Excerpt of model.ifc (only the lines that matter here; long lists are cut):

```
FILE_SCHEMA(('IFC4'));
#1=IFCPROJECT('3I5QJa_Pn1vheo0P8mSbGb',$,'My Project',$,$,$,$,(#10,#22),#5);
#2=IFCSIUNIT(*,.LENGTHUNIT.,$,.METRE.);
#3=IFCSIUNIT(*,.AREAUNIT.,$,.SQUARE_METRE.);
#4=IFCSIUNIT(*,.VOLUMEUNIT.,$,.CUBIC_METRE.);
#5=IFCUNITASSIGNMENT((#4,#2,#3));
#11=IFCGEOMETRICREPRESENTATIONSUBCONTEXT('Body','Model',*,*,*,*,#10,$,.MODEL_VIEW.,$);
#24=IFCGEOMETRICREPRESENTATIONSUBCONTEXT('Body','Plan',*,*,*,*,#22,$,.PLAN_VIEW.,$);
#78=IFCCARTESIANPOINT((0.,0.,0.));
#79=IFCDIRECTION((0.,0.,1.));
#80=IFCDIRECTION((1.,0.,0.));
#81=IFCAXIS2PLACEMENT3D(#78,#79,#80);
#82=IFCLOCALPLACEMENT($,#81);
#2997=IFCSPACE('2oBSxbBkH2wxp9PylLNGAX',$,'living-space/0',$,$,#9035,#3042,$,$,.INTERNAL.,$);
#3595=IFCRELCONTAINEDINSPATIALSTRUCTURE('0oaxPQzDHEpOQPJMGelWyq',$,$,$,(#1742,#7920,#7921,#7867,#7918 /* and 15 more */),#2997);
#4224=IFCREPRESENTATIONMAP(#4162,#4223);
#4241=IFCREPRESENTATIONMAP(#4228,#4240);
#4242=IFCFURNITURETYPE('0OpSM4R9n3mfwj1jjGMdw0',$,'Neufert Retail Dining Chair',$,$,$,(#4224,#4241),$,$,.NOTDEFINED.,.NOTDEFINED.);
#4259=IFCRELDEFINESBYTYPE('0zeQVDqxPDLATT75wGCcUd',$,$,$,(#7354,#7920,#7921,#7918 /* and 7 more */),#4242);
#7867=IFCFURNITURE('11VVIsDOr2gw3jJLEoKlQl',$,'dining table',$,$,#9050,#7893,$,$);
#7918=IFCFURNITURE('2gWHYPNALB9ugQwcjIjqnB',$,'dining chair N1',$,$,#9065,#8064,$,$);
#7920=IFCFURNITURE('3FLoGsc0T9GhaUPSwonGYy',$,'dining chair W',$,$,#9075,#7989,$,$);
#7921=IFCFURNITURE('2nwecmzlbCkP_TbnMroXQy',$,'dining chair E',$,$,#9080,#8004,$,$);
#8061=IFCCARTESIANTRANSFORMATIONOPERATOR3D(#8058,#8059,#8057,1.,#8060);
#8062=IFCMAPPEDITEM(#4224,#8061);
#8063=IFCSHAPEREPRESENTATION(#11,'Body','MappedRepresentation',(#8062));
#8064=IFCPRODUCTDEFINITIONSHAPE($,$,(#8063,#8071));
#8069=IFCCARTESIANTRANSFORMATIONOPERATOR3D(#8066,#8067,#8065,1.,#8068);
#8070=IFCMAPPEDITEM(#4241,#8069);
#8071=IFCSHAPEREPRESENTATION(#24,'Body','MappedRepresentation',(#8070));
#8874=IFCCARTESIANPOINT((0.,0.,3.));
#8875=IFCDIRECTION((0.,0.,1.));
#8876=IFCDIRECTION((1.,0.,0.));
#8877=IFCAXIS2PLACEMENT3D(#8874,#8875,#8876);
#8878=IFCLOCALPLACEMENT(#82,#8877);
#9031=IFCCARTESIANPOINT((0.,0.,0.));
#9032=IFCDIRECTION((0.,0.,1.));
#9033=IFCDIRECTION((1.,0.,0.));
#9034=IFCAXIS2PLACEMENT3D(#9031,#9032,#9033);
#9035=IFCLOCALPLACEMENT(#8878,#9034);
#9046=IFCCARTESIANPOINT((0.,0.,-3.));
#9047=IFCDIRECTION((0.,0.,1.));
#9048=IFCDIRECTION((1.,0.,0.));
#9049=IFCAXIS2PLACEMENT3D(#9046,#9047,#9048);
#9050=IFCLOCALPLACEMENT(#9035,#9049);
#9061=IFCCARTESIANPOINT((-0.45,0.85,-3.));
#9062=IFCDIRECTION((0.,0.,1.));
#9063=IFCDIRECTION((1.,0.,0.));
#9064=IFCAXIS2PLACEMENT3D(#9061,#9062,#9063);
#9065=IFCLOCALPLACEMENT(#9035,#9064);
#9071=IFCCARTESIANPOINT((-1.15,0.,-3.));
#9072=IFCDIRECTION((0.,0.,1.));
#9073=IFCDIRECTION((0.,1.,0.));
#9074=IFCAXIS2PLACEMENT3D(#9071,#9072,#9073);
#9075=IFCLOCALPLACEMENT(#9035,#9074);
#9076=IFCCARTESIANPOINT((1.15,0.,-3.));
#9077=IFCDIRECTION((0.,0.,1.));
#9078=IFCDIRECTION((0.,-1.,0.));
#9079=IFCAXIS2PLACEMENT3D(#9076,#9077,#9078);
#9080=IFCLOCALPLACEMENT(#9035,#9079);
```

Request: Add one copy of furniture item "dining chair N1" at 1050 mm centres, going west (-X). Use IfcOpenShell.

```python
import numpy as np
import ifcopenshell
import ifcopenshell.api.geometry
import ifcopenshell.api.root
import ifcopenshell.util.element
import ifcopenshell.util.placement
import ifcopenshell.util.unit

model = ifcopenshell.open("model.ifc")
unit_scale = ifcopenshell.util.unit.calculate_unit_scale(model)

source = model.by_id(7918)
base = ifcopenshell.util.placement.get_local_placement(source.ObjectPlacement)
step = np.array([-1.0, 0.0, 0.0]) * 1.05 / unit_scale

for i in range(1, 2):
    copy = ifcopenshell.api.root.copy_class(model, product=source)
    copy.Representation = ifcopenshell.util.element.copy_deep(
        model, source.Representation, exclude=["IfcGeometricRepresentationContext", "IfcRepresentationMap"]
    )
    matrix = base.copy()
    matrix[:3, 3] += i * step
    print("added at", matrix[:3, 3].round(3) + 0.0)
    ifcopenshell.api.geometry.edit_object_placement(model, product=copy, matrix=matrix, is_si=False)

model.write("model_updated.ifc")
```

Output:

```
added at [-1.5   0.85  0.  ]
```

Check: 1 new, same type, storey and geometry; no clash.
